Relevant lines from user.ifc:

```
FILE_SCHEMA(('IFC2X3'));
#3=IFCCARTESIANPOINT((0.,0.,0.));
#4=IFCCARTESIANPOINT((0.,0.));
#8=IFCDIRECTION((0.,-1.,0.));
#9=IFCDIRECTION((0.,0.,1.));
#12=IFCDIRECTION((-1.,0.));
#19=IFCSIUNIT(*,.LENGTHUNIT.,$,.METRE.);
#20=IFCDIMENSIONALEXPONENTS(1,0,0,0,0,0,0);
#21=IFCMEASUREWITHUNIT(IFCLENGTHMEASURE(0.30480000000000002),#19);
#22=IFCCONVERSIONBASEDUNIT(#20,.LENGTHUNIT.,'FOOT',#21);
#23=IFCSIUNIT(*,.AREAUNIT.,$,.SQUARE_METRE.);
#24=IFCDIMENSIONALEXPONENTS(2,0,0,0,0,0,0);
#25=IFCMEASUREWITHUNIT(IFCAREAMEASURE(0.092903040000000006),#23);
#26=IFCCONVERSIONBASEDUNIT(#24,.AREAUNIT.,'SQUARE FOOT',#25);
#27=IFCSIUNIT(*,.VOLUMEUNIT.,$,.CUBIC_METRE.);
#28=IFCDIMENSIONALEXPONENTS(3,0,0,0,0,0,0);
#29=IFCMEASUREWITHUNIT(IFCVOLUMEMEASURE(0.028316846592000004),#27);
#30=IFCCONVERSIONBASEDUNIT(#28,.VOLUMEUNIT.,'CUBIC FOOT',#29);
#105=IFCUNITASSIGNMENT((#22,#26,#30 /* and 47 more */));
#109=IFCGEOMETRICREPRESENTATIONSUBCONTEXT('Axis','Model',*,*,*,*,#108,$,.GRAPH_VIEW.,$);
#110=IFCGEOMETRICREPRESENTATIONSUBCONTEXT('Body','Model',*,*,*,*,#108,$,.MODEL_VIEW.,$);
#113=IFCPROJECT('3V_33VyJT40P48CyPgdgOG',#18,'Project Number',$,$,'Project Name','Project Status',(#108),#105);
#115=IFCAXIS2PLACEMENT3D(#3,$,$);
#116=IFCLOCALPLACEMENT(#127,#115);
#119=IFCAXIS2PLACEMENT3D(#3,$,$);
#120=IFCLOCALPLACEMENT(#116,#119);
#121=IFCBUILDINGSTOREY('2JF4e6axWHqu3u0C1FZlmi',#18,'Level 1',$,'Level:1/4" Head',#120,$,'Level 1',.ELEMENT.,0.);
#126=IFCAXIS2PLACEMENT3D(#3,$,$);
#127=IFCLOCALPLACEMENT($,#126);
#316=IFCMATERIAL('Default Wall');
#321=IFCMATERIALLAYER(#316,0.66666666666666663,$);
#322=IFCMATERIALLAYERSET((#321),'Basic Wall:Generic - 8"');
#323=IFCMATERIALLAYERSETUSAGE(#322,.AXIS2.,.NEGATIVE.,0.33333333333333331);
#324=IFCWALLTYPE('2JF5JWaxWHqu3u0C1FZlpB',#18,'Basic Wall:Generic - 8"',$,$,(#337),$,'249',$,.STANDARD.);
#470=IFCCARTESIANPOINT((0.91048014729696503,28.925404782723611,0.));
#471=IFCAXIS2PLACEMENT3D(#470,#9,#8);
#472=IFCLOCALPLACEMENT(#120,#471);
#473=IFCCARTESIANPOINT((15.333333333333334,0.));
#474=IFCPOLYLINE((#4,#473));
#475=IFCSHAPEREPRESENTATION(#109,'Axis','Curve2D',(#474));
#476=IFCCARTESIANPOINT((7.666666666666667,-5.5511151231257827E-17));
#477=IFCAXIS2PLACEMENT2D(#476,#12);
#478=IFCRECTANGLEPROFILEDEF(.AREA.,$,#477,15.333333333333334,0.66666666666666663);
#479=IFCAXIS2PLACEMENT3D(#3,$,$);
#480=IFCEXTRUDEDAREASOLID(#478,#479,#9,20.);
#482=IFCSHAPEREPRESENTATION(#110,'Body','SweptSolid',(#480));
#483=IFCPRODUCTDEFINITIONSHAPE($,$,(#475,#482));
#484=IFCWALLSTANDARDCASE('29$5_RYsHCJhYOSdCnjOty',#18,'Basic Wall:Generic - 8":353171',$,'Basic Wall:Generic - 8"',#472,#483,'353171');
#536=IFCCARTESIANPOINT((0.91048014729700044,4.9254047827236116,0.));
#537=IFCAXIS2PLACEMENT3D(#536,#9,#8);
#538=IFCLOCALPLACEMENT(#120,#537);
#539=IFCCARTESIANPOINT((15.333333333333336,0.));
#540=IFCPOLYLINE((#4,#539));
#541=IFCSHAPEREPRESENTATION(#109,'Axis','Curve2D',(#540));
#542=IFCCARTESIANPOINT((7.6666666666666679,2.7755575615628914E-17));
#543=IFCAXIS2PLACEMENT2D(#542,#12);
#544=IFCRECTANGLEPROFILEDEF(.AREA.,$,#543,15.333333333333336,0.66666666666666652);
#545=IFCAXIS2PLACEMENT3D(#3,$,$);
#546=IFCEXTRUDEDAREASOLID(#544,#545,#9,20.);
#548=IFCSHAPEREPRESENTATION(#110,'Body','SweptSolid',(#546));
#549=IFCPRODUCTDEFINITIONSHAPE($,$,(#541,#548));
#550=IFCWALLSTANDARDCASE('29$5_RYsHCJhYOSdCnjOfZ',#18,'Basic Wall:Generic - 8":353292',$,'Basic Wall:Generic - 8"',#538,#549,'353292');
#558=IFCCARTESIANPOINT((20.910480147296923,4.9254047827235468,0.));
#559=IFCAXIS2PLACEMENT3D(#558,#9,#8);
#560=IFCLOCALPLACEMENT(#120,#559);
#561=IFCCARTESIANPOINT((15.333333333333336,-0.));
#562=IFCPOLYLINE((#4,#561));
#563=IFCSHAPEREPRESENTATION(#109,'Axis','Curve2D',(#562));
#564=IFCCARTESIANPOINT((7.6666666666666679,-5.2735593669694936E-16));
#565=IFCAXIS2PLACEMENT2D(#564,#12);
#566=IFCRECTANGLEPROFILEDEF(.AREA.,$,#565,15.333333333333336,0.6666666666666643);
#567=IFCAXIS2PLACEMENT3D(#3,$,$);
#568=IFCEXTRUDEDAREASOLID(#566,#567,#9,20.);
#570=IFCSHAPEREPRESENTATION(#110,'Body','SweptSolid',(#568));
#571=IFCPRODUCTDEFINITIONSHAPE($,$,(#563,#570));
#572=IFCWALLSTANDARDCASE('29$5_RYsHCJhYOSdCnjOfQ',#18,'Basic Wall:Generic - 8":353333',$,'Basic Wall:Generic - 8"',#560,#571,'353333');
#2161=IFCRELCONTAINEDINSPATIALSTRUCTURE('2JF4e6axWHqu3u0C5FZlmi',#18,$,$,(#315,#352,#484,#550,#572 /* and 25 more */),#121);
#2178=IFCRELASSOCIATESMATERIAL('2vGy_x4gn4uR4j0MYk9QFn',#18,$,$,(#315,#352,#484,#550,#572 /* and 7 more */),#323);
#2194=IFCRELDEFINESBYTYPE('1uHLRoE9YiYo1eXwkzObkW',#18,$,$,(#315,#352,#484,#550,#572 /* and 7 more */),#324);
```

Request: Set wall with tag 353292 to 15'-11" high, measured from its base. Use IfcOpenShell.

```python
import ifcopenshell
import ifcopenshell.geom
import ifcopenshell.util.representation
import ifcopenshell.util.shape
import ifcopenshell.util.unit

model = ifcopenshell.open("user.ifc")
unit_scale = ifcopenshell.util.unit.calculate_unit_scale(model)
settings = ifcopenshell.geom.settings()


def volume(element):
    """Net volume in cubic metres, openings subtracted."""
    shape = ifcopenshell.geom.create_shape(settings, element)
    return ifcopenshell.util.shape.get_volume(shape.geometry)


wall = model.by_guid("29$5_RYsHCJhYOSdCnjOfZ")
before = volume(wall)

body = ifcopenshell.util.representation.get_representation(wall, "Model", "Body")
solid = body.Items[0]
old_height = solid.Depth
solid.Depth = 191 * 0.0254 / unit_scale
after = volume(wall)

print(f"height {old_height:g} -> {solid.Depth:g}, volume {before:.3f} -> {after:.3f} m3")

model.write("user_updated.ifc")
```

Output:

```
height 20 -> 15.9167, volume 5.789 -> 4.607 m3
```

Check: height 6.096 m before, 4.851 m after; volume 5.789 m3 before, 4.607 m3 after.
